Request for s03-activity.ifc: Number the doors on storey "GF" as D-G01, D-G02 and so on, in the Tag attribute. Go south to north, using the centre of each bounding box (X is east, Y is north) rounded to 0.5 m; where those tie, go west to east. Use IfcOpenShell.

First a look at what the model holds.

```python
import ifcopenshell
import ifcopenshell.util.element
import ifcopenshell.util.placement

model = ifcopenshell.open("s03-activity.ifc")
print(model.schema)
storey = next(s for s in model.by_type("IfcBuildingStorey") if s.Name == "GF")
doors = [e for e in ifcopenshell.util.element.get_decomposition(storey) if e.is_a("IfcDoor")]
for e in sorted(doors, key=lambda e: e.id()):
    origin = ifcopenshell.util.placement.get_local_placement(e.ObjectPlacement)[:3, 3]
    print(e.id(), e.Tag, e.Name, origin.round(2) + 0.0, sep=" | ")
```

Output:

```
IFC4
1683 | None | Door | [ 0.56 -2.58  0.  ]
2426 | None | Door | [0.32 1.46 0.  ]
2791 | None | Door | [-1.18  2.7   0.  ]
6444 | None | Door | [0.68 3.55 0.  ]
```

```python
import ifcopenshell
import ifcopenshell.geom
import ifcopenshell.util.element
import ifcopenshell.util.shape

model = ifcopenshell.open("s03-activity.ifc")
settings = ifcopenshell.geom.settings()
settings.set("use-world-coords", True)


def centre(element):
    shape = ifcopenshell.geom.create_shape(settings, element)
    return ifcopenshell.util.shape.get_bbox_centroid(shape.geometry)


storey = next(s for s in model.by_type("IfcBuildingStorey") if s.Name == "GF")
doors = [e for e in ifcopenshell.util.element.get_decomposition(storey) if e.is_a("IfcDoor")]

# Insertion points can sit at a corner or the storey origin, so sort by the geometry (in metres).
centres = {e: centre(e) for e in doors}
doors.sort(key=lambda e: (round(centres[e][1] / 0.5), centres[e][0]))

for i, e in enumerate(doors, start=1):
    number = f"D-G{i:02d}"
    e.Tag = number
    print(e.id(), number)

model.write("s03-activity_rev.ifc")
```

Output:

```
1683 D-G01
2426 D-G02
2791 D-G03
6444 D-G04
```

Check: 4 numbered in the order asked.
